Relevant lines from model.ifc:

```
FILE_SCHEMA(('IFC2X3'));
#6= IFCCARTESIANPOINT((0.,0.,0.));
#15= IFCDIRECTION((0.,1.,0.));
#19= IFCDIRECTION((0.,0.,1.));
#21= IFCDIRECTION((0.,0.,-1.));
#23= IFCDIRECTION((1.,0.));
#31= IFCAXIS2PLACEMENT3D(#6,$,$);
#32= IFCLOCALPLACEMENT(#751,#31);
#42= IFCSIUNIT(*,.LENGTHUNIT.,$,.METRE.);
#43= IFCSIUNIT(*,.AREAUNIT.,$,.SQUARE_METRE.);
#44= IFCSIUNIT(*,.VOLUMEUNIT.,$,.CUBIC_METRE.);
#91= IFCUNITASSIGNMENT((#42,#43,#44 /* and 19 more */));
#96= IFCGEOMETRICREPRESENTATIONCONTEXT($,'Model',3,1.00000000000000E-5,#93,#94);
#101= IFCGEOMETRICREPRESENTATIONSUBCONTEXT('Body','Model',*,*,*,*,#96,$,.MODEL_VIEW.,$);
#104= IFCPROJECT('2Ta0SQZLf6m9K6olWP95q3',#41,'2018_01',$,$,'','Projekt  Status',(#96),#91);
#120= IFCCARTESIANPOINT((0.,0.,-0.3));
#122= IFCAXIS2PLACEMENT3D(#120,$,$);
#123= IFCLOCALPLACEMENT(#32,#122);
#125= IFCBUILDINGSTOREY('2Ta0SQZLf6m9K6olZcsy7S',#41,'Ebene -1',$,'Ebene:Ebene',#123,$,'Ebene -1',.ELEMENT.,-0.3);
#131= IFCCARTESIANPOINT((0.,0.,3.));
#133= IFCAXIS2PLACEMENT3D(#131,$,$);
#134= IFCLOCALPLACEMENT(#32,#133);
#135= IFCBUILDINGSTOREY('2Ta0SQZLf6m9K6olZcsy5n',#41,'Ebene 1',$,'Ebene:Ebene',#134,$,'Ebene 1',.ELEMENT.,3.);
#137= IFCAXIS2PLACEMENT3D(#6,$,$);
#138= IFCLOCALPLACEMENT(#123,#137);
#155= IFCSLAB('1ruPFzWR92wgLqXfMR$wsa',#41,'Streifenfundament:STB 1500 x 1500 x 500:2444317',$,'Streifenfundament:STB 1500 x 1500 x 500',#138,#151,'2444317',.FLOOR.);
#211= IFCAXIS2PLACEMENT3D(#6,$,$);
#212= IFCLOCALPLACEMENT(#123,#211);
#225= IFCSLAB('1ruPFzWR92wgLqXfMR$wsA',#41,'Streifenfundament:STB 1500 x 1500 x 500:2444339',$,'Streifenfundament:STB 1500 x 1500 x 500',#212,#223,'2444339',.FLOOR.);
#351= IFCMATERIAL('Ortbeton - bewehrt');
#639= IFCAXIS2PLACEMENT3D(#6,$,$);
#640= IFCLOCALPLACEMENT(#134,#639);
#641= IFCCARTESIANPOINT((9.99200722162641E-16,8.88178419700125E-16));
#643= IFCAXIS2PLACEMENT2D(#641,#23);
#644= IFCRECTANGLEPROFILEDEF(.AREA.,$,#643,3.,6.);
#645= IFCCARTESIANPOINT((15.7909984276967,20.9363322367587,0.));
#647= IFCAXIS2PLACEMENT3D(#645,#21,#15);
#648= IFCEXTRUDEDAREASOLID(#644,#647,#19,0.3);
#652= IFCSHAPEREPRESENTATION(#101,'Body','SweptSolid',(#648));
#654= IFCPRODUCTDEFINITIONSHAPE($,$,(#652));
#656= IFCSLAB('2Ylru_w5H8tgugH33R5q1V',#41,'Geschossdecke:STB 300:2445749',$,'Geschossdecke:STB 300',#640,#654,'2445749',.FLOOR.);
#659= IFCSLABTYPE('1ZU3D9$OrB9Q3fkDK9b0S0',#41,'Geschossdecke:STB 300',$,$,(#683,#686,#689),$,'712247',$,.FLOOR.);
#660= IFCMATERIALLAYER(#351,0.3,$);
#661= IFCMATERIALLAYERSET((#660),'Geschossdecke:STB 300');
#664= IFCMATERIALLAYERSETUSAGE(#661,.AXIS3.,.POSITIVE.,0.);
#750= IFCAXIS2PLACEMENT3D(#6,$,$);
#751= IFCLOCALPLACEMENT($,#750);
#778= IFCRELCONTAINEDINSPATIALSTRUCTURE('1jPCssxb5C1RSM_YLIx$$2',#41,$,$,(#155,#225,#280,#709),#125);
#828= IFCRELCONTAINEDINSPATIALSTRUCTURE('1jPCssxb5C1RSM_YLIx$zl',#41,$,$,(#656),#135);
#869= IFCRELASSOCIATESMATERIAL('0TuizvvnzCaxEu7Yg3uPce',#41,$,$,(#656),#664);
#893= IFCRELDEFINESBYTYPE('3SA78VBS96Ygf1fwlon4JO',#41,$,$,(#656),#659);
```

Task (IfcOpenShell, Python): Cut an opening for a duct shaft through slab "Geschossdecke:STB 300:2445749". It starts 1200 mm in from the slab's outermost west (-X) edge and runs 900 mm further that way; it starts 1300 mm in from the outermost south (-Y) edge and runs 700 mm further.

```python
import numpy as np
import ifcopenshell
import ifcopenshell.api.feature
import ifcopenshell.api.geometry
import ifcopenshell.api.root
import ifcopenshell.geom
import ifcopenshell.util.placement
import ifcopenshell.util.representation
import ifcopenshell.util.shape
import ifcopenshell.util.unit

model = ifcopenshell.open("model.ifc")
unit_scale = ifcopenshell.util.unit.calculate_unit_scale(model)
settings = ifcopenshell.geom.settings()


def volume(element):
    """Net volume in cubic metres, openings subtracted."""
    shape = ifcopenshell.geom.create_shape(settings, element)
    return ifcopenshell.util.shape.get_volume(shape.geometry)


slab = model.by_id(656)
before = volume(slab)

# Extent in the slab's own axes, in metres. The edges named are its -X and -Y sides.
slab_shape = ifcopenshell.geom.create_shape(settings, slab)
vertices = ifcopenshell.util.shape.get_vertices(slab_shape.geometry)
x_min, y_min, bottom = vertices.min(axis=0)
top = vertices[:, 2].max()

opening = ifcopenshell.api.root.create_entity(model, ifc_class="IfcOpeningElement", name="Duct shaft opening")
context = ifcopenshell.util.representation.get_context(model, "Model", "Body", "MODEL_VIEW")
width, depth = 0.9, 0.7
outline = [(0.0, 0.0), (width, 0.0), (width, depth), (0.0, depth), (0.0, 0.0)]
# Overshoot both faces by 50 mm so the cut is clean.
shape = ifcopenshell.api.geometry.add_slab_representation(
    model, context=context, depth=top - bottom + 0.1, polyline=outline
)
ifcopenshell.api.geometry.assign_representation(model, product=opening, representation=shape)

matrix = ifcopenshell.util.placement.get_local_placement(slab.ObjectPlacement)
matrix[:, 3] = matrix @ np.append(np.array([x_min + 1.2, y_min + 1.3, bottom - 0.05]) / unit_scale, 1.0)
ifcopenshell.api.geometry.edit_object_placement(model, product=opening, matrix=matrix, is_si=False)
ifcopenshell.api.feature.add_feature(model, feature=opening, element=slab)

after = volume(slab)

print(f"slab volume {before:.3f} -> {after:.3f} m3")

model.write("model_v2.ifc")
```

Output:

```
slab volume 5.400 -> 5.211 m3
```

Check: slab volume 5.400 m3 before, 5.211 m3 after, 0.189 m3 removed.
